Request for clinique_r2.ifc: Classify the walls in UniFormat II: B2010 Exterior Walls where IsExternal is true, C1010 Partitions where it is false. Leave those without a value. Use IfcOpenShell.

First a look at what the model holds.

```python
import ifcopenshell
import ifcopenshell.util.element

model = ifcopenshell.open("clinique_r2.ifc")
print(model.schema)
print("classifications:", [c.Name for c in model.by_type("IfcClassification")])
values = [ifcopenshell.util.element.get_pset(e, "Pset_WallCommon", "IsExternal") for e in model.by_type("IfcWall")]
for value in (True, False, None):
    print("IsExternal", value, values.count(value))
```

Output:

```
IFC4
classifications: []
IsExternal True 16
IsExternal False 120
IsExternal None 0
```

```python
import ifcopenshell
import ifcopenshell.api.classification
import ifcopenshell.util.element

model = ifcopenshell.open("clinique_r2.ifc")

system = ifcopenshell.api.classification.add_classification(model, classification="UniFormat II")

walls = model.by_type("IfcWall")
external = {e: ifcopenshell.util.element.get_pset(e, "Pset_WallCommon", "IsExternal") for e in walls}
for flag, code, name in ((True, "B2010", "Exterior Walls"), (False, "C1010", "Partitions")):
    products = [e for e in walls if external[e] is flag]
    ifcopenshell.api.classification.add_reference(
        model, products=products, classification=system, identification=code, name=name
    )
    print(code, len(products))

model.write("clinique_r2_edited.ifc")
```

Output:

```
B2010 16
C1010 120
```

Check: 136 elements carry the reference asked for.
